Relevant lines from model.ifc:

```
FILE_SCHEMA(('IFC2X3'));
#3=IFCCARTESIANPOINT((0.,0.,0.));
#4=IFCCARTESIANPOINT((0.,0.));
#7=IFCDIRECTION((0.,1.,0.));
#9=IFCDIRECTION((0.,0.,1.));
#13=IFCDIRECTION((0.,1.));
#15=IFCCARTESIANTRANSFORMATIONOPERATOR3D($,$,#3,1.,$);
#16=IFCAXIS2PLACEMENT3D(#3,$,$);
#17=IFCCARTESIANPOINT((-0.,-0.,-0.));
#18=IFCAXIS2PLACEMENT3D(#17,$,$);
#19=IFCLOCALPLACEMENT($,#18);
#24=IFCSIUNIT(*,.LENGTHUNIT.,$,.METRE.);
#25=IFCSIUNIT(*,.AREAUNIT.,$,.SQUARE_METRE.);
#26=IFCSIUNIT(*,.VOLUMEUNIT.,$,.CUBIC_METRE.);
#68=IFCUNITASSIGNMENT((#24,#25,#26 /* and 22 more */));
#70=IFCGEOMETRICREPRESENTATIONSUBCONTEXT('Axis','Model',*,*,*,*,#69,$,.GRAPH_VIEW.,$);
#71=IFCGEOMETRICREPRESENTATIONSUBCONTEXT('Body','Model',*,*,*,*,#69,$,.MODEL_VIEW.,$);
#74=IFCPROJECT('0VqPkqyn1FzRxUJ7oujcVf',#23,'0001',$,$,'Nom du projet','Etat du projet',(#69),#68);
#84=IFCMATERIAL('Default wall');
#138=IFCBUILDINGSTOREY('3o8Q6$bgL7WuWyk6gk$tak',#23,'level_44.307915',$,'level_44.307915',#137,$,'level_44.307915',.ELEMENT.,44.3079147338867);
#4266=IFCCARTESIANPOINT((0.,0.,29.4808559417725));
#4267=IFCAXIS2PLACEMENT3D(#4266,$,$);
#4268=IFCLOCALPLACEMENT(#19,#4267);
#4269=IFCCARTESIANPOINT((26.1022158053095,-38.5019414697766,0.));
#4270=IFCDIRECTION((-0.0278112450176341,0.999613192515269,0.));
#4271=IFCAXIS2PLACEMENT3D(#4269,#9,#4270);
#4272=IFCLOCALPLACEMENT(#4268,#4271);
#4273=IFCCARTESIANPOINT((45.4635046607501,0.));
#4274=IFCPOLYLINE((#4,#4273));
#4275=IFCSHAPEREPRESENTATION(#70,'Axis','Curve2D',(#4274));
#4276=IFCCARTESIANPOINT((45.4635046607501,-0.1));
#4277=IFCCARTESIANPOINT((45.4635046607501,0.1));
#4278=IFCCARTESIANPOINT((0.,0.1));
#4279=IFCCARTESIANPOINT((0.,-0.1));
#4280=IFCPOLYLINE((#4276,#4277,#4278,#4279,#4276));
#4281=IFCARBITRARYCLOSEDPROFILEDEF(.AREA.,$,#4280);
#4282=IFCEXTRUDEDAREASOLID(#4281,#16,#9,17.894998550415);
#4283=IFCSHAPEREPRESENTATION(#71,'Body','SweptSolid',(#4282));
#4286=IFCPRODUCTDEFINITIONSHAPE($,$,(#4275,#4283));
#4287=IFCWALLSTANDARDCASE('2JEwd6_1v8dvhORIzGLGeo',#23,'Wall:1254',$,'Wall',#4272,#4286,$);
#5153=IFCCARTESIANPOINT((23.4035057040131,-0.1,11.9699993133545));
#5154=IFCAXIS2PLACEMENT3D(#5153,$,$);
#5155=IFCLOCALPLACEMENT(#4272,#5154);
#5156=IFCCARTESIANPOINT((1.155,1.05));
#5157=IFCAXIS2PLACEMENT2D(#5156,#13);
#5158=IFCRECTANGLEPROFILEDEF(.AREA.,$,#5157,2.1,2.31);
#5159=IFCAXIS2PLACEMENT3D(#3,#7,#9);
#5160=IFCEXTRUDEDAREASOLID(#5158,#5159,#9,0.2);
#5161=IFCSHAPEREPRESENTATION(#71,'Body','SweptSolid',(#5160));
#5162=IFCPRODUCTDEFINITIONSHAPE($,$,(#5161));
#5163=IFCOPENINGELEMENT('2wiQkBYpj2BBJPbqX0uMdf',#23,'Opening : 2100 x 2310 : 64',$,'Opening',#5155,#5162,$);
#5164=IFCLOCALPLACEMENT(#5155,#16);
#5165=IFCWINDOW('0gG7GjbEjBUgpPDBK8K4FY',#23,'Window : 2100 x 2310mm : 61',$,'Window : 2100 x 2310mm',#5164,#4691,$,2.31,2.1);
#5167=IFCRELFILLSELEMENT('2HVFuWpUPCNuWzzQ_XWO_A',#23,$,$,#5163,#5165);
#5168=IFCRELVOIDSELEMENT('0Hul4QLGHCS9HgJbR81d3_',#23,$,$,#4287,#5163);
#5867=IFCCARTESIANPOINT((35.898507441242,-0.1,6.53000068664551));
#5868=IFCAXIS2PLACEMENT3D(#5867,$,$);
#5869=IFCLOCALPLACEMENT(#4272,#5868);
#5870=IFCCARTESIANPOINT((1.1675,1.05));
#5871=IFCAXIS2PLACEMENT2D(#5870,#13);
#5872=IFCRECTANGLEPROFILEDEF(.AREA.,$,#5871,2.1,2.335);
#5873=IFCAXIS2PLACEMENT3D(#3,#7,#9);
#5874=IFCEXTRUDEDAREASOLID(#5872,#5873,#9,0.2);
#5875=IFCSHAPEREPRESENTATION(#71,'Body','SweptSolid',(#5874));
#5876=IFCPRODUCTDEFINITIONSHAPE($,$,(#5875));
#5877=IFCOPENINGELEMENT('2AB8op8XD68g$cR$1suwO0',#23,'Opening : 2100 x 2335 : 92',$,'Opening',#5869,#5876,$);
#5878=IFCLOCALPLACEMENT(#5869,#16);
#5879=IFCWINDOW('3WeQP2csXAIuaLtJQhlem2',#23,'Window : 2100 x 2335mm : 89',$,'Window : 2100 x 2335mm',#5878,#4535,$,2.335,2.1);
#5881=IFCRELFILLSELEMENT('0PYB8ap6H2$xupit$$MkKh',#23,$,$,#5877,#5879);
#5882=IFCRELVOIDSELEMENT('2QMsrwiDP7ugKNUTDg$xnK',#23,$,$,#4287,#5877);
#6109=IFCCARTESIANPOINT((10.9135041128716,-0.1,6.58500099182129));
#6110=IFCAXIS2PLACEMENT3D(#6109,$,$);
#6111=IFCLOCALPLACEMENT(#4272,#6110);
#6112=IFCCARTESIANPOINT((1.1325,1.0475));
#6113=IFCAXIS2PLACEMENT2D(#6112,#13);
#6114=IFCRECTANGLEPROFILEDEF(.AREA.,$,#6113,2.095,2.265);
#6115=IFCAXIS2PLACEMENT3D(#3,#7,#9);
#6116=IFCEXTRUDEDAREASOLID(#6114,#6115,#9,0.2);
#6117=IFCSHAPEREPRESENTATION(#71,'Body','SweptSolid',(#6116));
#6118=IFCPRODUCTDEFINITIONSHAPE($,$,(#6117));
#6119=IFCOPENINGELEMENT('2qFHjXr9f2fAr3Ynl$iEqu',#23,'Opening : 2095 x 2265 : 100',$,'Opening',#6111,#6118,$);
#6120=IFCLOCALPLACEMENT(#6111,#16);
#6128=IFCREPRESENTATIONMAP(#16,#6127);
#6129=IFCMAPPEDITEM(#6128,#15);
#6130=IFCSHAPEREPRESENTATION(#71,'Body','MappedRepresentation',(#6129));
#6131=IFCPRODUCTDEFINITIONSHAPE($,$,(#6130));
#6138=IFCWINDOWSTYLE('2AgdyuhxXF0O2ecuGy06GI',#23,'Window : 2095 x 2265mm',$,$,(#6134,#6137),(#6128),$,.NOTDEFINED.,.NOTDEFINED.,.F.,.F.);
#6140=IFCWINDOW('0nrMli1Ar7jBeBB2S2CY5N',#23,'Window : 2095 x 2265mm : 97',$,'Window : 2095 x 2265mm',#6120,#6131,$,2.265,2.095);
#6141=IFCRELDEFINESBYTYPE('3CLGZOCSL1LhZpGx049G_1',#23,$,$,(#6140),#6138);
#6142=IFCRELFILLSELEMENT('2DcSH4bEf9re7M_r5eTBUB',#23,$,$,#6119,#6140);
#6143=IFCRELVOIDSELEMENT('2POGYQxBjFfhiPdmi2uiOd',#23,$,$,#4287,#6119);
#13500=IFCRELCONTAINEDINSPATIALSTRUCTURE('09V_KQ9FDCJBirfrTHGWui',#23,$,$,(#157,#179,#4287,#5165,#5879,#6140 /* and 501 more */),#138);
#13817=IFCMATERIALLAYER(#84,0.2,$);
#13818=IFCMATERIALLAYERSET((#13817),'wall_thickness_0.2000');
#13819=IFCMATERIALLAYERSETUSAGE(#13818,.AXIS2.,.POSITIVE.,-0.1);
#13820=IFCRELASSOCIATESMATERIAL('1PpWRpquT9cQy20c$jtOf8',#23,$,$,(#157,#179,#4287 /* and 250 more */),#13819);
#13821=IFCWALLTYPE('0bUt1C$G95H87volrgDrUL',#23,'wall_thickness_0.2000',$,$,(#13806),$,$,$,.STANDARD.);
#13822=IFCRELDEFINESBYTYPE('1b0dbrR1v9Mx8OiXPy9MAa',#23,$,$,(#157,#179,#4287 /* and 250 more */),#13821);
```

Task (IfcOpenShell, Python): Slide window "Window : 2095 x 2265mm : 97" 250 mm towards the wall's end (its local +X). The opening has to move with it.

```python
import ifcopenshell
import ifcopenshell.api.geometry
import ifcopenshell.util.placement
import ifcopenshell.util.unit

model = ifcopenshell.open("model.ifc")
unit_scale = ifcopenshell.util.unit.calculate_unit_scale(model)

window = model.by_id(6140)
opening = window.FillsVoids[0].RelatingOpeningElement
wall = opening.VoidsElements[0].RelatingBuildingElement

wall_matrix = ifcopenshell.util.placement.get_local_placement(wall.ObjectPlacement)
shift = wall_matrix[:3, 0] * 0.25 / unit_scale
before = ifcopenshell.util.placement.get_local_placement(window.ObjectPlacement)[:3, 3].copy()

# The window is placed relative to its opening, so it follows when the opening moves.
matrix = ifcopenshell.util.placement.get_local_placement(opening.ObjectPlacement)
matrix[:3, 3] += shift
ifcopenshell.api.geometry.edit_object_placement(
    model, product=opening, matrix=matrix, is_si=False, should_transform_children=True
)

after = ifcopenshell.util.placement.get_local_placement(window.ObjectPlacement)[:3, 3]
print("window moved by", (after - before).round(3) + 0.0)

model.write("model-out.ifc")
```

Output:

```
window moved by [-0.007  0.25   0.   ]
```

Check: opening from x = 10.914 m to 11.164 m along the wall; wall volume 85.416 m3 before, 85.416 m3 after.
